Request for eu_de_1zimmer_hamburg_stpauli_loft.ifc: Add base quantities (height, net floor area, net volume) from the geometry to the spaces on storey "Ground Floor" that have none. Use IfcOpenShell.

First a look at what the model holds.

```python
import ifcopenshell
import ifcopenshell.util.element
import ifcopenshell.util.unit

model = ifcopenshell.open("eu_de_1zimmer_hamburg_stpauli_loft.ifc")
print(model.schema)
for unit_type in ("LENGTHUNIT", "AREAUNIT", "VOLUMEUNIT"):
    print(unit_type, ifcopenshell.util.unit.calculate_unit_scale(model, unit_type))
storey = next(s for s in model.by_type("IfcBuildingStorey") if s.Name == "Ground Floor")
spaces = [e for e in ifcopenshell.util.element.get_decomposition(storey) if e.is_a("IfcSpace")]
for e in sorted(spaces, key=lambda e: e.id()):
    print(e.id(), e.is_a(), e.Name, list(ifcopenshell.util.element.get_psets(e, qtos_only=True)), sep=" | ")
```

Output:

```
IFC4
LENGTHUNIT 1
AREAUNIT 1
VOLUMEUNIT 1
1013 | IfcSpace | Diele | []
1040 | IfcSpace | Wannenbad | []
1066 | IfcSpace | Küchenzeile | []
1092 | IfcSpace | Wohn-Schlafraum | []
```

```python
import ifcopenshell
import ifcopenshell.api.pset
import ifcopenshell.geom
import ifcopenshell.util.element
import ifcopenshell.util.shape
import ifcopenshell.util.unit

model = ifcopenshell.open("eu_de_1zimmer_hamburg_stpauli_loft.ifc")
unit_scale = ifcopenshell.util.unit.calculate_unit_scale(model)
area_scale = ifcopenshell.util.unit.calculate_unit_scale(model, "AREAUNIT")
volume_scale = ifcopenshell.util.unit.calculate_unit_scale(model, "VOLUMEUNIT")
settings = ifcopenshell.geom.settings()

storey = next(s for s in model.by_type("IfcBuildingStorey") if s.Name == "Ground Floor")
spaces = [e for e in ifcopenshell.util.element.get_decomposition(storey) if e.is_a("IfcSpace")]

for e in sorted(spaces, key=lambda e: e.id()):
    if ifcopenshell.util.element.get_psets(e, qtos_only=True, should_inherit=False):
        continue
    # Geometry comes back in metres, in the element's own axes.
    shape = ifcopenshell.geom.create_shape(settings, e)
    values = {
        "Height": ifcopenshell.util.shape.get_z(shape.geometry) / unit_scale,
        "NetFloorArea": ifcopenshell.util.shape.get_footprint_area(shape.geometry) / area_scale,
        "NetVolume": ifcopenshell.util.shape.get_volume(shape.geometry) / volume_scale,
    }
    qto = ifcopenshell.api.pset.add_qto(model, product=e, name="Qto_SpaceBaseQuantities")
    ifcopenshell.api.pset.edit_qto(model, qto=qto, properties=values)
    print(e.id(), {k: round(v, 3) for k, v in values.items()})

model.write("eu_de_1zimmer_hamburg_stpauli_loft_rev.ifc")
```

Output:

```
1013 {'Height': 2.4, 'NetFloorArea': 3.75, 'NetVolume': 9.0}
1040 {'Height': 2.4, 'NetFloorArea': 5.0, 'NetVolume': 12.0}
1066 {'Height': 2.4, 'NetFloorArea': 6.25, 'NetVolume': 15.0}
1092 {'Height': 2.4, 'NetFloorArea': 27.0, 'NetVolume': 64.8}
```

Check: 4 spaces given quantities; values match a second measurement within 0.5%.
